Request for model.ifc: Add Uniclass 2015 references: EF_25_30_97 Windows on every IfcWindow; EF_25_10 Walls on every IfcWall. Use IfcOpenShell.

First a look at what the model holds.

```python
import ifcopenshell

model = ifcopenshell.open("model.ifc")
print(model.schema)
print("classifications:", [c.Name for c in model.by_type("IfcClassification")])
for ifc_class in ("IfcDoor", "IfcRoof", "IfcStair", "IfcWall", "IfcWindow"):
    print(ifc_class, len(model.by_type(ifc_class)))
```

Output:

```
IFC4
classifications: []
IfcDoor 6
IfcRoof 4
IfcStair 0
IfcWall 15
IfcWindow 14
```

```python
import ifcopenshell
import ifcopenshell.api.classification

model = ifcopenshell.open("model.ifc")

system = ifcopenshell.api.classification.add_classification(model, classification="Uniclass 2015")

codes = {
    "IfcWindow": ("EF_25_30_97", "Windows"),
    "IfcWall": ("EF_25_10", "Walls"),
}
for ifc_class, (code, name) in codes.items():
    products = model.by_type(ifc_class)
    ifcopenshell.api.classification.add_reference(
        model, products=products, classification=system, identification=code, name=name
    )
    print(code, len(products))

model.write("model-out.ifc")
```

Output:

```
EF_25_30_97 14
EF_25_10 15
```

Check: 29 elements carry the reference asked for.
